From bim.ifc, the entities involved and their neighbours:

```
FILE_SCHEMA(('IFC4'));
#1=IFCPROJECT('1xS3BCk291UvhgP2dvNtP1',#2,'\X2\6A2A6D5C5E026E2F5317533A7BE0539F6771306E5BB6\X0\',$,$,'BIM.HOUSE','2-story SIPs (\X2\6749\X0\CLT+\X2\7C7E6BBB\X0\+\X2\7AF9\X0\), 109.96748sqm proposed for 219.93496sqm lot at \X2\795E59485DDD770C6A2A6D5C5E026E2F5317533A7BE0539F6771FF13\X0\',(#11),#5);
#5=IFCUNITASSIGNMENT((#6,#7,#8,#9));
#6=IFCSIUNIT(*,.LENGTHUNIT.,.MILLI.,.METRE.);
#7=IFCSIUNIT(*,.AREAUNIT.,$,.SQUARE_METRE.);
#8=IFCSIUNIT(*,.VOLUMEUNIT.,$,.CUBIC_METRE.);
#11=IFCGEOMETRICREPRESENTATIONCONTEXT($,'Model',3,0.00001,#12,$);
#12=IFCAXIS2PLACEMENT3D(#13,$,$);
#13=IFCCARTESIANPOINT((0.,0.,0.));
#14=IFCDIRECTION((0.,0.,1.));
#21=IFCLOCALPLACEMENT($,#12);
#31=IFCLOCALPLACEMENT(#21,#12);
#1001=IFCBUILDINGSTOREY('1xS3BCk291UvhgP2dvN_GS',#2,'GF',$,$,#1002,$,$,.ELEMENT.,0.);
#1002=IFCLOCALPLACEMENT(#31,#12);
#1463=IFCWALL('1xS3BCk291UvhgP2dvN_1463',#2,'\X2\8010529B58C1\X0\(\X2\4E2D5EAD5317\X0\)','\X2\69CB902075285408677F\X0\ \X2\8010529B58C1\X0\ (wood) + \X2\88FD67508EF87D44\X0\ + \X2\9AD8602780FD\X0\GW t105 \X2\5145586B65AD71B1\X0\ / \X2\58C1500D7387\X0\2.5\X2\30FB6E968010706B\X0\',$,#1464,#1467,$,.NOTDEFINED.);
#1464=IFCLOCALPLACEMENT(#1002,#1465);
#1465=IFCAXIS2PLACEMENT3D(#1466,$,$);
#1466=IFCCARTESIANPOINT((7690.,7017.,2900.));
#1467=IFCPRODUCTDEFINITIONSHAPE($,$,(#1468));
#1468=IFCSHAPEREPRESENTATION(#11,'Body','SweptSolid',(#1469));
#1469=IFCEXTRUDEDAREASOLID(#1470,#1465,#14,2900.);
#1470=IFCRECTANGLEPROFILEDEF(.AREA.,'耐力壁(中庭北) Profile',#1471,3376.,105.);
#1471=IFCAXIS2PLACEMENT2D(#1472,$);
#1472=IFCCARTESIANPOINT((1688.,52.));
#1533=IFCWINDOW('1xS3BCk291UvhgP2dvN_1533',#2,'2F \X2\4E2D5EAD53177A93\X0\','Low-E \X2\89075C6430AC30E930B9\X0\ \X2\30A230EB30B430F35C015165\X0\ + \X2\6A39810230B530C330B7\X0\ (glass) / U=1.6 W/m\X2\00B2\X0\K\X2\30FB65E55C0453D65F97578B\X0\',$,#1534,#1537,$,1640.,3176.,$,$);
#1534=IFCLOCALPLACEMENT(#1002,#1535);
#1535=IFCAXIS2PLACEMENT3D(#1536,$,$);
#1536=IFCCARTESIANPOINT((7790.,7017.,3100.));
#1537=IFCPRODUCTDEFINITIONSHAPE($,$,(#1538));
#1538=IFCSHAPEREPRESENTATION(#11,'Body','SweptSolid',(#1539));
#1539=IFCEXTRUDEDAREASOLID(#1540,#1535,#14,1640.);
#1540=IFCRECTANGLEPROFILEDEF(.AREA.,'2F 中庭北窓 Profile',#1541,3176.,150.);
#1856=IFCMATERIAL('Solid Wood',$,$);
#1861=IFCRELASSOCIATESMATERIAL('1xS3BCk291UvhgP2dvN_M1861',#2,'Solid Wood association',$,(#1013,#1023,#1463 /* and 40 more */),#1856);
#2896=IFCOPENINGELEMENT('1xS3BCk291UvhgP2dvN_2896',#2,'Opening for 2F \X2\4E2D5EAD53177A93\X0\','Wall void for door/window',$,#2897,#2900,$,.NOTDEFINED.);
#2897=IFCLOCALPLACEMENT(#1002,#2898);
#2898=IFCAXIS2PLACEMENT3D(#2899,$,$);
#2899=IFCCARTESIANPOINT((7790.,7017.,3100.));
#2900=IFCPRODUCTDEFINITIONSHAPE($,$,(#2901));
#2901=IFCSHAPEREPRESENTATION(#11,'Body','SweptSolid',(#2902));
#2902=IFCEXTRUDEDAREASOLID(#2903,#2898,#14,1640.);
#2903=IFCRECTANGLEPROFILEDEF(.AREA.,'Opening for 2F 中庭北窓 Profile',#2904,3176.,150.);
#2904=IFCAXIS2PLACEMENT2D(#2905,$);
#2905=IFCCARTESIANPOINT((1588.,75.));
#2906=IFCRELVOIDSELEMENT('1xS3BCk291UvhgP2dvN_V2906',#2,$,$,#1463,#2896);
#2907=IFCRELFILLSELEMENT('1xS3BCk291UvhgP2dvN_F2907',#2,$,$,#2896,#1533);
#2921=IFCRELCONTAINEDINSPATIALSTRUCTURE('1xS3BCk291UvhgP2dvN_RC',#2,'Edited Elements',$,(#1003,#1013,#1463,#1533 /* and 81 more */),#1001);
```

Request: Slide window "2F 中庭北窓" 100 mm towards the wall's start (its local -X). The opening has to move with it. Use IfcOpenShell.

```python
import ifcopenshell
import ifcopenshell.api.geometry
import ifcopenshell.util.placement
import ifcopenshell.util.unit

model = ifcopenshell.open("bim.ifc")
unit_scale = ifcopenshell.util.unit.calculate_unit_scale(model)

window = model.by_guid("1xS3BCk291UvhgP2dvN_1533")
opening = window.FillsVoids[0].RelatingOpeningElement
wall = opening.VoidsElements[0].RelatingBuildingElement

wall_matrix = ifcopenshell.util.placement.get_local_placement(wall.ObjectPlacement)
shift = wall_matrix[:3, 0] * -0.1 / unit_scale
before = ifcopenshell.util.placement.get_local_placement(window.ObjectPlacement)[:3, 3].copy()

# The window is not placed relative to its opening, so move both.
for product in (opening, window):
    matrix = ifcopenshell.util.placement.get_local_placement(product.ObjectPlacement)
    matrix[:3, 3] += shift
    ifcopenshell.api.geometry.edit_object_placement(model, product=product, matrix=matrix, is_si=False)

after = ifcopenshell.util.placement.get_local_placement(window.ObjectPlacement)[:3, 3]
print("window moved by", (after - before).round(3) + 0.0)

model.write("bim-out.ifc")
```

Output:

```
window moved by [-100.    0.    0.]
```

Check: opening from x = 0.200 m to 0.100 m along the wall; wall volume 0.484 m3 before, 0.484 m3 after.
